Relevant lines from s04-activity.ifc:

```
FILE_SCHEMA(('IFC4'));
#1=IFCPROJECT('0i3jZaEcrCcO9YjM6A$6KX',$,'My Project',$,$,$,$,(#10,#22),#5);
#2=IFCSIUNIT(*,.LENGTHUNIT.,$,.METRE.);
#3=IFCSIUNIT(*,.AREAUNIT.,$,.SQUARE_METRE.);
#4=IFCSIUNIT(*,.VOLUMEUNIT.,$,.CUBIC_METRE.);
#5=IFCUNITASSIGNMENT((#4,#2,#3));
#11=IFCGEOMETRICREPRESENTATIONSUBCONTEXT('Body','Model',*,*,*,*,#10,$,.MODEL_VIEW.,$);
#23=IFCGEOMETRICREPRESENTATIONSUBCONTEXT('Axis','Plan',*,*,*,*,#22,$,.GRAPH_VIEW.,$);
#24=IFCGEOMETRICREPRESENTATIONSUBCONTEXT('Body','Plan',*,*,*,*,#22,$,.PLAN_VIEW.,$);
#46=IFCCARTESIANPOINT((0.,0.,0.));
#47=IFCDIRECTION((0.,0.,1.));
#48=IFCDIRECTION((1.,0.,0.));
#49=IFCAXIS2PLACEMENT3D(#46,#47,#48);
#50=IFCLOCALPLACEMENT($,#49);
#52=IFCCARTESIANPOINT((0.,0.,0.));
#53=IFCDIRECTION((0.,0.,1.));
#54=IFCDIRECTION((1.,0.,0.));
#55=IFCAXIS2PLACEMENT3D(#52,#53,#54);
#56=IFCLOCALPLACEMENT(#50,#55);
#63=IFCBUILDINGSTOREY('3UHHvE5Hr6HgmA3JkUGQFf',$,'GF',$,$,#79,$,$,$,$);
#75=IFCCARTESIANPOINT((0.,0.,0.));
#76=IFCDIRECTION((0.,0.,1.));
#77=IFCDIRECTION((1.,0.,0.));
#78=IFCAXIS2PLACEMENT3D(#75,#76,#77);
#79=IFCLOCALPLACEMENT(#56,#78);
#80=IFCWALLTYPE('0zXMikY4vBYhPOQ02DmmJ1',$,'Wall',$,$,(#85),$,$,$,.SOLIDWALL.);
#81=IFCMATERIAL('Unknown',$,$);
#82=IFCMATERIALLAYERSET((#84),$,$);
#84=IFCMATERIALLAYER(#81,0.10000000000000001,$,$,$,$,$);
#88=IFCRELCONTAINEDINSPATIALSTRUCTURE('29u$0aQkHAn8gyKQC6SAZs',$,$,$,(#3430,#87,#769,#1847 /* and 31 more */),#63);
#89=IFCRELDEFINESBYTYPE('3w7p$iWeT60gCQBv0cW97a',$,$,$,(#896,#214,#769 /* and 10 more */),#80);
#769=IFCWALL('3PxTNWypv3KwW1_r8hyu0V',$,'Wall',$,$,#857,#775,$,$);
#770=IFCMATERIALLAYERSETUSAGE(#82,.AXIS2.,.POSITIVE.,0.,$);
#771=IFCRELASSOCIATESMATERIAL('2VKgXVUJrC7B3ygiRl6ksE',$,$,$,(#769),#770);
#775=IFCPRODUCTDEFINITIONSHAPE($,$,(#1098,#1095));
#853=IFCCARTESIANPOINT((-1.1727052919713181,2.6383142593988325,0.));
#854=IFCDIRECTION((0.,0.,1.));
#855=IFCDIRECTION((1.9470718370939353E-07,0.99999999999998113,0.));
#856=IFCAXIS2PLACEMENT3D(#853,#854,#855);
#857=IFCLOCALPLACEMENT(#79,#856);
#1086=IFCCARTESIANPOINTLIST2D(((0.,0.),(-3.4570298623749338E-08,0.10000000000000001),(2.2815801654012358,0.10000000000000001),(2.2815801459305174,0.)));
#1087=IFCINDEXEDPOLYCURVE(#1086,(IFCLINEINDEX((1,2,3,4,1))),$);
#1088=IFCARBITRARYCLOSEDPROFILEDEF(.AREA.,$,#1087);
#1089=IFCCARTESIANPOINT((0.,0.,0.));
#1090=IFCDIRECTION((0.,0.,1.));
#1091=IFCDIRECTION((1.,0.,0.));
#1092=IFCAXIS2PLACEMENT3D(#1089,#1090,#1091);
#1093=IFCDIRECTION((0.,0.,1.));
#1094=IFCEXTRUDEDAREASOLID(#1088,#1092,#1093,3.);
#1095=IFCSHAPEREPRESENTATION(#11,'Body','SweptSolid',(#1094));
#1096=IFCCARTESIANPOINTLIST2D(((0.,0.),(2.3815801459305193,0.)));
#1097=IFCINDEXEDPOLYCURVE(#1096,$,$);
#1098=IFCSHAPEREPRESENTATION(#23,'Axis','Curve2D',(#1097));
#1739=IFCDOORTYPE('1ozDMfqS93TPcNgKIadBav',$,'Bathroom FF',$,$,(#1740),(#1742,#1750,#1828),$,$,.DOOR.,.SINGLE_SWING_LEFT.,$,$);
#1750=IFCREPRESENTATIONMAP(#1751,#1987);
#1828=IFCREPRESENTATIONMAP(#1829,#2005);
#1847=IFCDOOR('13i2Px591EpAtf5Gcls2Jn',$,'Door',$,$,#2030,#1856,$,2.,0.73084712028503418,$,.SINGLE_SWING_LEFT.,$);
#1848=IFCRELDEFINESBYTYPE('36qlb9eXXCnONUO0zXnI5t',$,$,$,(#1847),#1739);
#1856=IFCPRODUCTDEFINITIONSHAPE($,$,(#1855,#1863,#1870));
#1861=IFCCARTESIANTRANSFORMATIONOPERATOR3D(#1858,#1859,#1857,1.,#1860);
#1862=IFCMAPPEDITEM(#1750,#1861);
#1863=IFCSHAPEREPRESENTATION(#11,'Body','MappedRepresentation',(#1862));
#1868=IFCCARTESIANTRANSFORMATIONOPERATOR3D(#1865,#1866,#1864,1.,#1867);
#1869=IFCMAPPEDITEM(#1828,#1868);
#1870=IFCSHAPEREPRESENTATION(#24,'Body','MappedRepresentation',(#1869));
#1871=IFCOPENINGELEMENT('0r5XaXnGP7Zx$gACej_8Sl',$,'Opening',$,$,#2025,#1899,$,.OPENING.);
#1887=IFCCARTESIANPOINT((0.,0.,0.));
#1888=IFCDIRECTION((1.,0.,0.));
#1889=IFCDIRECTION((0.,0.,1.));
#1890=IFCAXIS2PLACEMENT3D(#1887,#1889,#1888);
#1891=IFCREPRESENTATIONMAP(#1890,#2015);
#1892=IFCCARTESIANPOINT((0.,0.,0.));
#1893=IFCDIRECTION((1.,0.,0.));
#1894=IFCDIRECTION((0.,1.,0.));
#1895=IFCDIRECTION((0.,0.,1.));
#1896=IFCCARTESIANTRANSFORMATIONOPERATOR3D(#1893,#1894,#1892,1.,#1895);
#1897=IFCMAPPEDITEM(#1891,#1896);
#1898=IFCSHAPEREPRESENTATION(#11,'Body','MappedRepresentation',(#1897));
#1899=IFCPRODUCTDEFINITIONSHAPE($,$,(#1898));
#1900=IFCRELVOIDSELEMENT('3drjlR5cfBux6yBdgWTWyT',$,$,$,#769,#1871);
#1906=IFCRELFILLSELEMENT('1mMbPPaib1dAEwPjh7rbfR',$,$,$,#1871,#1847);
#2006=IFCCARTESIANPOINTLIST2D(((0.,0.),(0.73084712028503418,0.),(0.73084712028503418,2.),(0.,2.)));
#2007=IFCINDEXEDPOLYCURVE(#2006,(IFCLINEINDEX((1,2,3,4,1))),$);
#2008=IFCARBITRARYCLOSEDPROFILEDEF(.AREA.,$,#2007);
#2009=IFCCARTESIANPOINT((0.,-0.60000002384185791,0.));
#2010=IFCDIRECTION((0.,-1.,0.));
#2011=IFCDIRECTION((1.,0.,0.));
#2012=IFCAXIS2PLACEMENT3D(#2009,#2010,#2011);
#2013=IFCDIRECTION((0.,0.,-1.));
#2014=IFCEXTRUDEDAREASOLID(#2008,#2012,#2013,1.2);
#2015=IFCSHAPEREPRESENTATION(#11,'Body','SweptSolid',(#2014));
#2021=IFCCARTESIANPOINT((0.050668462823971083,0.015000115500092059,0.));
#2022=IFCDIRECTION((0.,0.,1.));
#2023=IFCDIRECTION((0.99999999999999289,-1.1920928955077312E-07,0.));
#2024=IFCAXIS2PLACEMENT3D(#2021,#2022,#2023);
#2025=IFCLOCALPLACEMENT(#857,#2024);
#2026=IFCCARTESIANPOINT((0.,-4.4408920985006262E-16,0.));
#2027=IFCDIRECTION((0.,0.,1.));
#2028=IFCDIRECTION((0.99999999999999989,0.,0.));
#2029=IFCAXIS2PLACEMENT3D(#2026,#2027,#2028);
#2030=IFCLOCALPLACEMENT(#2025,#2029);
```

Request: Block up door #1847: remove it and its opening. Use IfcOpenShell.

```python
import ifcopenshell
import ifcopenshell.api.feature
import ifcopenshell.api.root
import ifcopenshell.geom
import ifcopenshell.util.shape

model = ifcopenshell.open("s04-activity.ifc")
settings = ifcopenshell.geom.settings()


def volume(element):
    """Net volume in cubic metres, openings subtracted."""
    shape = ifcopenshell.geom.create_shape(settings, element)
    return ifcopenshell.util.shape.get_volume(shape.geometry)


door = model.by_guid("13i2Px591EpAtf5Gcls2Jn")
opening = door.FillsVoids[0].RelatingOpeningElement
wall = opening.VoidsElements[0].RelatingBuildingElement
before = volume(wall)

ifcopenshell.api.root.remove_product(model, product=door)
ifcopenshell.api.feature.remove_feature(model, feature=opening)

after = volume(wall)

print(f"wall volume {before:.3f} -> {after:.3f} m3")

model.write("s04-activity_updated.ifc")
```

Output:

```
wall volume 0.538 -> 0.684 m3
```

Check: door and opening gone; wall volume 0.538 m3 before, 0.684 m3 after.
